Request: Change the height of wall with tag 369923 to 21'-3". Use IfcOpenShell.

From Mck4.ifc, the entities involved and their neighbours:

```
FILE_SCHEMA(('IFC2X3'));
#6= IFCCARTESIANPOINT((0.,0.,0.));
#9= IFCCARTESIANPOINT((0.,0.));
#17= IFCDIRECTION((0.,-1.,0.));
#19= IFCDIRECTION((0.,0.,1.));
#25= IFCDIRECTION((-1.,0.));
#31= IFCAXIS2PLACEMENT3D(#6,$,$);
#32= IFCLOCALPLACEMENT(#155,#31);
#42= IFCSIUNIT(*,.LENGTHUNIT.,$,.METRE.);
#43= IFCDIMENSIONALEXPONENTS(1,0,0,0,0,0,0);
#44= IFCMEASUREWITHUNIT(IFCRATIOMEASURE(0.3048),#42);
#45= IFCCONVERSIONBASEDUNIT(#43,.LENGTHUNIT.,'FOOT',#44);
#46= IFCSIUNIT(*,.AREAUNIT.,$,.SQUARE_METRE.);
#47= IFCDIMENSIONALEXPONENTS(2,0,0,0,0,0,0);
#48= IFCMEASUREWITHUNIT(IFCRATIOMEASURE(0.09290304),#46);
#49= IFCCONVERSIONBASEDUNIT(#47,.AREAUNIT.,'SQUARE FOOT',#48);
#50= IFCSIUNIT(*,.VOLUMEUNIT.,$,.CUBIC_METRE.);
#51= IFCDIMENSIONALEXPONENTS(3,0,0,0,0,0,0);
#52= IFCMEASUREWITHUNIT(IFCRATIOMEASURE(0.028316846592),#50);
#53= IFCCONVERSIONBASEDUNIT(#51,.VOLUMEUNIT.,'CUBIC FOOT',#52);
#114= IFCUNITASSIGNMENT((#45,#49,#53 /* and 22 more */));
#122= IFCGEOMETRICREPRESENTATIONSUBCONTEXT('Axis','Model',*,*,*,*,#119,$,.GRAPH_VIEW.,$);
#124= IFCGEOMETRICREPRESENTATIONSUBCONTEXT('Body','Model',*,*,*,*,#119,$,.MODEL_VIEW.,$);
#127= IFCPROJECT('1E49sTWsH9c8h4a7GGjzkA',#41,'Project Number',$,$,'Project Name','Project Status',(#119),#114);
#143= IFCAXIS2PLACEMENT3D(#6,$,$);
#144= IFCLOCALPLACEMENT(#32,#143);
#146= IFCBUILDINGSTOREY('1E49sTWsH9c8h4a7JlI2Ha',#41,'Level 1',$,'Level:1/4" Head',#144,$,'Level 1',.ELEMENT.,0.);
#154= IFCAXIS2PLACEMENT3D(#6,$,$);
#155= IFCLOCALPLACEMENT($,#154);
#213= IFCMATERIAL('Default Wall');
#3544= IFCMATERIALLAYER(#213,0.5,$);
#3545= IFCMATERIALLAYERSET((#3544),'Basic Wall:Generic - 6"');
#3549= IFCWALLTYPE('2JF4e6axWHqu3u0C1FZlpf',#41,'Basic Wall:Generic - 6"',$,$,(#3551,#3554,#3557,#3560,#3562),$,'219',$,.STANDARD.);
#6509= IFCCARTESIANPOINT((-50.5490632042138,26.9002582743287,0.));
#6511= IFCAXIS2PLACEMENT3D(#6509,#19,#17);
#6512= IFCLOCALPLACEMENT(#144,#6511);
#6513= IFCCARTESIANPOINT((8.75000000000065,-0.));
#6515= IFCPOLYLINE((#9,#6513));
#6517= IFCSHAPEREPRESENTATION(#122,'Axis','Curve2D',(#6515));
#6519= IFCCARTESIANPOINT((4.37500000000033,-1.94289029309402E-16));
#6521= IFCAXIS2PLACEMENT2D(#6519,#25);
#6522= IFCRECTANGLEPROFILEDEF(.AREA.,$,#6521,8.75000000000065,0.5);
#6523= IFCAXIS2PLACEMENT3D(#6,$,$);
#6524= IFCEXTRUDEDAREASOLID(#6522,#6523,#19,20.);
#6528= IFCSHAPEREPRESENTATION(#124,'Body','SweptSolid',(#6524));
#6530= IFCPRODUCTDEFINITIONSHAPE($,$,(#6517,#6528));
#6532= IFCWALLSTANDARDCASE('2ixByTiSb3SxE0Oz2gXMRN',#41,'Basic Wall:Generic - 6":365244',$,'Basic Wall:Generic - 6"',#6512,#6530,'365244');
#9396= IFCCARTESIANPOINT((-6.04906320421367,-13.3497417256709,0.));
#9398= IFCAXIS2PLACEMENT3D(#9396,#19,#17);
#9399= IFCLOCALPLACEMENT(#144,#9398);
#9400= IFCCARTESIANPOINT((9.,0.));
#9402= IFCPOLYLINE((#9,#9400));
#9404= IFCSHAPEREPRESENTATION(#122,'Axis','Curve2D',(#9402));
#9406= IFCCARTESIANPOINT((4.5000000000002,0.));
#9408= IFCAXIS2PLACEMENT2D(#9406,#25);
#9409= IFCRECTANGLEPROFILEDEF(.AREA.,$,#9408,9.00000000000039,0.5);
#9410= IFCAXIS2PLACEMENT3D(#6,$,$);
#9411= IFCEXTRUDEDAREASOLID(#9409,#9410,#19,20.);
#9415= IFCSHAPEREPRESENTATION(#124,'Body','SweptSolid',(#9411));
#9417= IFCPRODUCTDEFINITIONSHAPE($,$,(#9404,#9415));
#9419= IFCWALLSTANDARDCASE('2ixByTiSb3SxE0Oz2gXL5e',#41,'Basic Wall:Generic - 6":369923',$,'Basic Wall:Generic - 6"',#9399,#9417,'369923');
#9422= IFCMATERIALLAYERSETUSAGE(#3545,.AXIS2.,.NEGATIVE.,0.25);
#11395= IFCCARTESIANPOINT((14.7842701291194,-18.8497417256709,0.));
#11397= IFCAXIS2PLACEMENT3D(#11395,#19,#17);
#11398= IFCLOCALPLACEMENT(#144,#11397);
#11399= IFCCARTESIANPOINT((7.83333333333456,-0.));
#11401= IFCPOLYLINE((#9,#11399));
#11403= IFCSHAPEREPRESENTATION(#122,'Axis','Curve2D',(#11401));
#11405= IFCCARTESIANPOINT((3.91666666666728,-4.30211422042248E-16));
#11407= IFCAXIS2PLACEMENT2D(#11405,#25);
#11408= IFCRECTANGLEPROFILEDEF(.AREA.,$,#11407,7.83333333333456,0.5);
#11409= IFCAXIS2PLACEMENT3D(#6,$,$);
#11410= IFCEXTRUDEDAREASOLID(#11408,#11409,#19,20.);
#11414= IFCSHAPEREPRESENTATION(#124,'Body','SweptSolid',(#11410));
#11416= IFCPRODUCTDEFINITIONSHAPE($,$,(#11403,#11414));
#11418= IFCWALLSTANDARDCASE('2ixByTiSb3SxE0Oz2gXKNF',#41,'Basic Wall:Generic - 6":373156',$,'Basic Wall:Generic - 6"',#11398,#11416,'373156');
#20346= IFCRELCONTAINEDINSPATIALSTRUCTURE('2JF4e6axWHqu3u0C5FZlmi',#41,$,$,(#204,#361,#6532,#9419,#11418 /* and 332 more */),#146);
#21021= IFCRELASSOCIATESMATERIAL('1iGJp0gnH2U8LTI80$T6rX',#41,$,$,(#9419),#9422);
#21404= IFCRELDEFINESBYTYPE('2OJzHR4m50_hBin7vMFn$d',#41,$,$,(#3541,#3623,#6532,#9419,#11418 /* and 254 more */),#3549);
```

```python
import ifcopenshell
import ifcopenshell.geom
import ifcopenshell.util.representation
import ifcopenshell.util.shape
import ifcopenshell.util.unit

model = ifcopenshell.open("Mck4.ifc")
unit_scale = ifcopenshell.util.unit.calculate_unit_scale(model)
settings = ifcopenshell.geom.settings()


def volume(element):
    """Net volume in cubic metres, openings subtracted."""
    shape = ifcopenshell.geom.create_shape(settings, element)
    return ifcopenshell.util.shape.get_volume(shape.geometry)


wall = model.by_id(9419)
before = volume(wall)

body = ifcopenshell.util.representation.get_representation(wall, "Model", "Body")
solid = body.Items[0]
old_height = solid.Depth
solid.Depth = 255 * 0.0254 / unit_scale
after = volume(wall)

print(f"height {old_height:g} -> {solid.Depth:g}, volume {before:.3f} -> {after:.3f} m3")

model.write("Mck4_edited.ifc")
```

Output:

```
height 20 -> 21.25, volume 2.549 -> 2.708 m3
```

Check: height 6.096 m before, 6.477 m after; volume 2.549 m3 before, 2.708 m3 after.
